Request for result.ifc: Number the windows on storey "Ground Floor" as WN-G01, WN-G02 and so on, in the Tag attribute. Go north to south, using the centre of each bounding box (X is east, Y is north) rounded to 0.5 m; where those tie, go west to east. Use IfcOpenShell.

First a look at what the model holds.

```python
import ifcopenshell
import ifcopenshell.util.element
import ifcopenshell.util.placement

model = ifcopenshell.open("result.ifc")
print(model.schema)
storey = next(s for s in model.by_type("IfcBuildingStorey") if s.Name == "Ground Floor")
windows = [e for e in ifcopenshell.util.element.get_decomposition(storey) if e.is_a("IfcWindow")]
for e in sorted(windows, key=lambda e: e.id()):
    origin = ifcopenshell.util.placement.get_local_placement(e.ObjectPlacement)[:3, 3]
    print(e.id(), e.Tag, e.Name, origin.round(2) + 0.0, sep=" | ")
```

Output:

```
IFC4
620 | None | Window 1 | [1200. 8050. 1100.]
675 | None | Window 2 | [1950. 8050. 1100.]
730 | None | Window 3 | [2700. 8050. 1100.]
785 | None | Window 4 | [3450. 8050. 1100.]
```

```python
import ifcopenshell
import ifcopenshell.geom
import ifcopenshell.util.element
import ifcopenshell.util.shape

model = ifcopenshell.open("result.ifc")
settings = ifcopenshell.geom.settings()
settings.set("use-world-coords", True)


def centre(element):
    shape = ifcopenshell.geom.create_shape(settings, element)
    return ifcopenshell.util.shape.get_bbox_centroid(shape.geometry)


storey = next(s for s in model.by_type("IfcBuildingStorey") if s.Name == "Ground Floor")
windows = [e for e in ifcopenshell.util.element.get_decomposition(storey) if e.is_a("IfcWindow")]

# Insertion points can sit at a corner or the storey origin, so sort by the geometry (in metres).
centres = {e: centre(e) for e in windows}
windows.sort(key=lambda e: (-round(centres[e][1] / 0.5), centres[e][0]))

for i, e in enumerate(windows, start=1):
    number = f"WN-G{i:02d}"
    e.Tag = number
    print(e.id(), number)

model.write("result_updated.ifc")
```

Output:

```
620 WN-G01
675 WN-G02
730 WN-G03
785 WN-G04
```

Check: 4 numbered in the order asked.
